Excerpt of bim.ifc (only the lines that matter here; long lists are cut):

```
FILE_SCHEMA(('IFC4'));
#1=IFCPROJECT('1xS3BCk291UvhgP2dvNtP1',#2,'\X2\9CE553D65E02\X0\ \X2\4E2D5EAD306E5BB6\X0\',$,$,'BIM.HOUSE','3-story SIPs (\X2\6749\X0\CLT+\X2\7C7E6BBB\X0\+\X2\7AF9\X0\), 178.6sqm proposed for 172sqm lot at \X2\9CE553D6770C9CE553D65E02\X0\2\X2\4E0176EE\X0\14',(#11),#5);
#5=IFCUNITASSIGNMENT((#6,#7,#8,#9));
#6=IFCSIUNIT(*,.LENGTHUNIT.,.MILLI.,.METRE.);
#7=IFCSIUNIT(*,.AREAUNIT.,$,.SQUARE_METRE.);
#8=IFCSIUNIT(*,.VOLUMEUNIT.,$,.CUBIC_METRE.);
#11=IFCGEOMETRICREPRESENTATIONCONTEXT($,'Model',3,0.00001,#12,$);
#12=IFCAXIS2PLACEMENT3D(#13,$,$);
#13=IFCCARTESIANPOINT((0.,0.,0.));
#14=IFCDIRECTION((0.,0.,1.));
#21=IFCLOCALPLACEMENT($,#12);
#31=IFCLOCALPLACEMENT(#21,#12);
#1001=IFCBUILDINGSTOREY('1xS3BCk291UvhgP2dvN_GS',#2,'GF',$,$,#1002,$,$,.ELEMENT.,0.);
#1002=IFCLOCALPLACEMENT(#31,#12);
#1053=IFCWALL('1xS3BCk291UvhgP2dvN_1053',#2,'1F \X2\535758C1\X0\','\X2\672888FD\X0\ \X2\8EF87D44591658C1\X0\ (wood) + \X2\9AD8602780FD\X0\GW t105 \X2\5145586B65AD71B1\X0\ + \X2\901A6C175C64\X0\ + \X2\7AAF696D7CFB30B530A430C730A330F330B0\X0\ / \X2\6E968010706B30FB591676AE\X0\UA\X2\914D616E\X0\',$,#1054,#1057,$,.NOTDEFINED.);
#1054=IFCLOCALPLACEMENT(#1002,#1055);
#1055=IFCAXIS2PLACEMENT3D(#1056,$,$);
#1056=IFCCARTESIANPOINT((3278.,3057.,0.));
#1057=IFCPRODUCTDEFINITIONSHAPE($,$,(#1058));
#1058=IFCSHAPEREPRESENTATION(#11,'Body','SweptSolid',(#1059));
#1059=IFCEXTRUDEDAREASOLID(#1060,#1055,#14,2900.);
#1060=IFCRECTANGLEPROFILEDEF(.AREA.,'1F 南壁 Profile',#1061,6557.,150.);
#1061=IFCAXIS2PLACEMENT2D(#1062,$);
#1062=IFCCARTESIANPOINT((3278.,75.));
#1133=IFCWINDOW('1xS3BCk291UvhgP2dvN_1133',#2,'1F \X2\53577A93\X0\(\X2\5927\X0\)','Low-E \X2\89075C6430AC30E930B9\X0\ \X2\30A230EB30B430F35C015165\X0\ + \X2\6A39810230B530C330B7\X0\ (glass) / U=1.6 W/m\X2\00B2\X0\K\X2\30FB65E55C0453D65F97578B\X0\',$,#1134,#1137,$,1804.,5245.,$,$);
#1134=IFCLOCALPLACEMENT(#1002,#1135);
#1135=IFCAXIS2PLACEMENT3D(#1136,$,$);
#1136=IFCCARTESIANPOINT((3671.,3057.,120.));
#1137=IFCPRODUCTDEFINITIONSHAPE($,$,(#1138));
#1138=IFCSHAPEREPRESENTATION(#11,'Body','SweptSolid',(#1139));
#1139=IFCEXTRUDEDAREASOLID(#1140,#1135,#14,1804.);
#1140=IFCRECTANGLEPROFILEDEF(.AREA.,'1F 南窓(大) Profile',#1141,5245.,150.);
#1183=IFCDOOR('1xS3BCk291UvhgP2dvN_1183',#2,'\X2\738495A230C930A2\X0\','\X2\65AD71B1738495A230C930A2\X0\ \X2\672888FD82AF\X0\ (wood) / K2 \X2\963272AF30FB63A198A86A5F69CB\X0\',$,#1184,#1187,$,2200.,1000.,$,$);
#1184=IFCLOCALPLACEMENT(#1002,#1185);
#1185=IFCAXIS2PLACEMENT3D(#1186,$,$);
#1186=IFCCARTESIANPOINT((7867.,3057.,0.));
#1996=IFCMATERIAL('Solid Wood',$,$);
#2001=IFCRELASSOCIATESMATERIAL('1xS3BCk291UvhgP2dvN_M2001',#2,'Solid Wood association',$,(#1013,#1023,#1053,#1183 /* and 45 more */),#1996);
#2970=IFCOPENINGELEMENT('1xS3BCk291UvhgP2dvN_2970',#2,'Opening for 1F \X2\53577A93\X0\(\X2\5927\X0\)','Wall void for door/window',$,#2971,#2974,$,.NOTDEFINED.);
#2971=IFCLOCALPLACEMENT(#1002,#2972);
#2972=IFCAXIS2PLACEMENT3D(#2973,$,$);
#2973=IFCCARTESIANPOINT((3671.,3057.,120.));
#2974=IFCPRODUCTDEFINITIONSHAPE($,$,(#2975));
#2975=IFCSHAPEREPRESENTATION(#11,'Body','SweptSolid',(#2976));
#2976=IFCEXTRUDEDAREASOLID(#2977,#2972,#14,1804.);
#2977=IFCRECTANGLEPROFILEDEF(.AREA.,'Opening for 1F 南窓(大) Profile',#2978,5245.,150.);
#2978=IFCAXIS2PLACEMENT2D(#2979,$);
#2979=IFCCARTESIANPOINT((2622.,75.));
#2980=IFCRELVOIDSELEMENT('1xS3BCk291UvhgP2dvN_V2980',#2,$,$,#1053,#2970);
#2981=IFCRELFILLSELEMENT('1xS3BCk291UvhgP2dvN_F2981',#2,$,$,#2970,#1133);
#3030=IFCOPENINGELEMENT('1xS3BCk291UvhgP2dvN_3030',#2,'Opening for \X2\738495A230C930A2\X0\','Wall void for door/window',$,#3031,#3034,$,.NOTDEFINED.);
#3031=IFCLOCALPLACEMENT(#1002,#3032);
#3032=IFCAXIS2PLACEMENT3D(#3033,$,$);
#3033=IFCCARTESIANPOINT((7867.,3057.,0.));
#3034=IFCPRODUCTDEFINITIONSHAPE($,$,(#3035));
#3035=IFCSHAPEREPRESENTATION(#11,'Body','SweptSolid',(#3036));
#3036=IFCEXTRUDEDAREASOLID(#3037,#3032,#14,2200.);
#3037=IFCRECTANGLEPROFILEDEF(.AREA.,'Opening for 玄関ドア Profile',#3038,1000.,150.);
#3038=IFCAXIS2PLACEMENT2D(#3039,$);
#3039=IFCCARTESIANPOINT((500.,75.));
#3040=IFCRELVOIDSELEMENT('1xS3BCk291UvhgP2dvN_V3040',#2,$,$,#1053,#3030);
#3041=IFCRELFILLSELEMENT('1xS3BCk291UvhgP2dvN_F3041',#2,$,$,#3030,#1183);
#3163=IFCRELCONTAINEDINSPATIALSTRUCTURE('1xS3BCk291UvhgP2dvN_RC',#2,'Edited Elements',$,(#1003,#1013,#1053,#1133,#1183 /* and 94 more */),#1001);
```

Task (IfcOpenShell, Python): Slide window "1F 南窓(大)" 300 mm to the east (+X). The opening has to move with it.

```python
import ifcopenshell
import ifcopenshell.api.geometry
import ifcopenshell.util.placement
import ifcopenshell.util.unit

model = ifcopenshell.open("bim.ifc")
unit_scale = ifcopenshell.util.unit.calculate_unit_scale(model)

window = model.by_id(1133)
opening = window.FillsVoids[0].RelatingOpeningElement
wall = opening.VoidsElements[0].RelatingBuildingElement

wall_matrix = ifcopenshell.util.placement.get_local_placement(wall.ObjectPlacement)
shift = wall_matrix[:3, 0] * 0.3 / unit_scale
before = ifcopenshell.util.placement.get_local_placement(window.ObjectPlacement)[:3, 3].copy()

# The window is not placed relative to its opening, so move both.
for product in (opening, window):
    matrix = ifcopenshell.util.placement.get_local_placement(product.ObjectPlacement)
    matrix[:3, 3] += shift
    ifcopenshell.api.geometry.edit_object_placement(model, product=product, matrix=matrix, is_si=False)

after = ifcopenshell.util.placement.get_local_placement(window.ObjectPlacement)[:3, 3]
print("window moved by", (after - before).round(3) + 0.0)

model.write("bim_updated.ifc")
```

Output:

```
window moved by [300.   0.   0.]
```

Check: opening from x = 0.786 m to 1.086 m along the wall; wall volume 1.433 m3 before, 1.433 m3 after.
